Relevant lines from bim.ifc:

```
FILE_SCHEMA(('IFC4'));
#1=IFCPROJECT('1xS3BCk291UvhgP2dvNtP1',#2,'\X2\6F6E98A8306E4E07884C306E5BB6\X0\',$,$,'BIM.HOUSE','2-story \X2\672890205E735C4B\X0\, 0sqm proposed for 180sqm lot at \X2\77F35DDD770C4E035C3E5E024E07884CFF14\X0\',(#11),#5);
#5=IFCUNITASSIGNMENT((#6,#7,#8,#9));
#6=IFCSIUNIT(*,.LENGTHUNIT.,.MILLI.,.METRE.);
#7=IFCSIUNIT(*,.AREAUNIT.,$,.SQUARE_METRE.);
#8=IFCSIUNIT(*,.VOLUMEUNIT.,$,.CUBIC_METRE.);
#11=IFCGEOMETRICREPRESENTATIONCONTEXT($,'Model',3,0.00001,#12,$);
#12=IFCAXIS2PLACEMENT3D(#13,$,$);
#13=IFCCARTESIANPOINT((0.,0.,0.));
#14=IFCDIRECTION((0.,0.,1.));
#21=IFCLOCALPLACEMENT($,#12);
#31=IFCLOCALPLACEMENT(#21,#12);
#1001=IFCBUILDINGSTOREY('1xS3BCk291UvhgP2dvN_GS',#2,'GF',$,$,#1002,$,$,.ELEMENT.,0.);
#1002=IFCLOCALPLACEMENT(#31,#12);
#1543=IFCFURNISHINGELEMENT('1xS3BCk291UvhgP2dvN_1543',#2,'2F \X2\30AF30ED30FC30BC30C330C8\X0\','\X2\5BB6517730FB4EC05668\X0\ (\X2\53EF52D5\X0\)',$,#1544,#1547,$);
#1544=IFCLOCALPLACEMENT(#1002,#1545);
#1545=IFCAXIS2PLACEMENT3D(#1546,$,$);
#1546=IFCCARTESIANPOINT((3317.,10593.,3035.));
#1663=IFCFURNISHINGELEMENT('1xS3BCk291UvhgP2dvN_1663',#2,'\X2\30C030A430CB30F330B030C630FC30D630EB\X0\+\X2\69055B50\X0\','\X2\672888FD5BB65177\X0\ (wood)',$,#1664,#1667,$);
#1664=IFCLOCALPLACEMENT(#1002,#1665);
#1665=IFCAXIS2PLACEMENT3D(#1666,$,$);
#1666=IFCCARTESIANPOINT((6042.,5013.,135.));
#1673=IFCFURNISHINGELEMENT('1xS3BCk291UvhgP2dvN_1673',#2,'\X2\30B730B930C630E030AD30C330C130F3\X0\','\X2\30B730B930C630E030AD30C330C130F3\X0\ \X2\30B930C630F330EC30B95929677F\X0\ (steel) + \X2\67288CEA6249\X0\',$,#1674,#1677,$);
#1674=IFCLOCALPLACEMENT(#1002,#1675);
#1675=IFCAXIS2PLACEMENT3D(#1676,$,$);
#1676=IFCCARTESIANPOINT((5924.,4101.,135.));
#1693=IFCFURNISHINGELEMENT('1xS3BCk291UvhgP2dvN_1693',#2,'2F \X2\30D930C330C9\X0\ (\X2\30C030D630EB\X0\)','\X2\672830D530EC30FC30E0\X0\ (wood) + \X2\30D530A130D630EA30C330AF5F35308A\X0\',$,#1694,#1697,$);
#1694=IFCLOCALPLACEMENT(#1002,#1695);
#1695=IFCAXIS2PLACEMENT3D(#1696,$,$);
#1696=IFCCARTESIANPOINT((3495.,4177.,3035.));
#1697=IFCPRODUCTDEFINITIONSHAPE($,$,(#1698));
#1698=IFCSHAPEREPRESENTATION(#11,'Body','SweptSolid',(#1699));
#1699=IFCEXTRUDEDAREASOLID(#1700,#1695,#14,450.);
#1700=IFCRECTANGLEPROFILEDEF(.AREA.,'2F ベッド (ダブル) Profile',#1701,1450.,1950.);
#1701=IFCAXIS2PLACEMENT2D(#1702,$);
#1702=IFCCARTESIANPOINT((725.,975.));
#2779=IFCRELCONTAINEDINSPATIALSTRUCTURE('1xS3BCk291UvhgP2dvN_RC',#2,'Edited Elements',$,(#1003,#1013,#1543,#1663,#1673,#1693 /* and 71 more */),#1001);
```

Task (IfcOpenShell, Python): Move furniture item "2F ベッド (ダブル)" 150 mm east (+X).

```python
import ifcopenshell
import ifcopenshell.api.geometry
import ifcopenshell.util.placement
import ifcopenshell.util.unit

model = ifcopenshell.open("bim.ifc")
unit_scale = ifcopenshell.util.unit.calculate_unit_scale(model)

item = model.by_id(1693)
matrix = ifcopenshell.util.placement.get_local_placement(item.ObjectPlacement)
matrix[0, 3] += 0.15 / unit_scale
ifcopenshell.api.geometry.edit_object_placement(model, product=item, matrix=matrix, is_si=False)

print(ifcopenshell.util.placement.get_local_placement(item.ObjectPlacement).round(3) + 0.0)

model.write("bim_v2.ifc")
```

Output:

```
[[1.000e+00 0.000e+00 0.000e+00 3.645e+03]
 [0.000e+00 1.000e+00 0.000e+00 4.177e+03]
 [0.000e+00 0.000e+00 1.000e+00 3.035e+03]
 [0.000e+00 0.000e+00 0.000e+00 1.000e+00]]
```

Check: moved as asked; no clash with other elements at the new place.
